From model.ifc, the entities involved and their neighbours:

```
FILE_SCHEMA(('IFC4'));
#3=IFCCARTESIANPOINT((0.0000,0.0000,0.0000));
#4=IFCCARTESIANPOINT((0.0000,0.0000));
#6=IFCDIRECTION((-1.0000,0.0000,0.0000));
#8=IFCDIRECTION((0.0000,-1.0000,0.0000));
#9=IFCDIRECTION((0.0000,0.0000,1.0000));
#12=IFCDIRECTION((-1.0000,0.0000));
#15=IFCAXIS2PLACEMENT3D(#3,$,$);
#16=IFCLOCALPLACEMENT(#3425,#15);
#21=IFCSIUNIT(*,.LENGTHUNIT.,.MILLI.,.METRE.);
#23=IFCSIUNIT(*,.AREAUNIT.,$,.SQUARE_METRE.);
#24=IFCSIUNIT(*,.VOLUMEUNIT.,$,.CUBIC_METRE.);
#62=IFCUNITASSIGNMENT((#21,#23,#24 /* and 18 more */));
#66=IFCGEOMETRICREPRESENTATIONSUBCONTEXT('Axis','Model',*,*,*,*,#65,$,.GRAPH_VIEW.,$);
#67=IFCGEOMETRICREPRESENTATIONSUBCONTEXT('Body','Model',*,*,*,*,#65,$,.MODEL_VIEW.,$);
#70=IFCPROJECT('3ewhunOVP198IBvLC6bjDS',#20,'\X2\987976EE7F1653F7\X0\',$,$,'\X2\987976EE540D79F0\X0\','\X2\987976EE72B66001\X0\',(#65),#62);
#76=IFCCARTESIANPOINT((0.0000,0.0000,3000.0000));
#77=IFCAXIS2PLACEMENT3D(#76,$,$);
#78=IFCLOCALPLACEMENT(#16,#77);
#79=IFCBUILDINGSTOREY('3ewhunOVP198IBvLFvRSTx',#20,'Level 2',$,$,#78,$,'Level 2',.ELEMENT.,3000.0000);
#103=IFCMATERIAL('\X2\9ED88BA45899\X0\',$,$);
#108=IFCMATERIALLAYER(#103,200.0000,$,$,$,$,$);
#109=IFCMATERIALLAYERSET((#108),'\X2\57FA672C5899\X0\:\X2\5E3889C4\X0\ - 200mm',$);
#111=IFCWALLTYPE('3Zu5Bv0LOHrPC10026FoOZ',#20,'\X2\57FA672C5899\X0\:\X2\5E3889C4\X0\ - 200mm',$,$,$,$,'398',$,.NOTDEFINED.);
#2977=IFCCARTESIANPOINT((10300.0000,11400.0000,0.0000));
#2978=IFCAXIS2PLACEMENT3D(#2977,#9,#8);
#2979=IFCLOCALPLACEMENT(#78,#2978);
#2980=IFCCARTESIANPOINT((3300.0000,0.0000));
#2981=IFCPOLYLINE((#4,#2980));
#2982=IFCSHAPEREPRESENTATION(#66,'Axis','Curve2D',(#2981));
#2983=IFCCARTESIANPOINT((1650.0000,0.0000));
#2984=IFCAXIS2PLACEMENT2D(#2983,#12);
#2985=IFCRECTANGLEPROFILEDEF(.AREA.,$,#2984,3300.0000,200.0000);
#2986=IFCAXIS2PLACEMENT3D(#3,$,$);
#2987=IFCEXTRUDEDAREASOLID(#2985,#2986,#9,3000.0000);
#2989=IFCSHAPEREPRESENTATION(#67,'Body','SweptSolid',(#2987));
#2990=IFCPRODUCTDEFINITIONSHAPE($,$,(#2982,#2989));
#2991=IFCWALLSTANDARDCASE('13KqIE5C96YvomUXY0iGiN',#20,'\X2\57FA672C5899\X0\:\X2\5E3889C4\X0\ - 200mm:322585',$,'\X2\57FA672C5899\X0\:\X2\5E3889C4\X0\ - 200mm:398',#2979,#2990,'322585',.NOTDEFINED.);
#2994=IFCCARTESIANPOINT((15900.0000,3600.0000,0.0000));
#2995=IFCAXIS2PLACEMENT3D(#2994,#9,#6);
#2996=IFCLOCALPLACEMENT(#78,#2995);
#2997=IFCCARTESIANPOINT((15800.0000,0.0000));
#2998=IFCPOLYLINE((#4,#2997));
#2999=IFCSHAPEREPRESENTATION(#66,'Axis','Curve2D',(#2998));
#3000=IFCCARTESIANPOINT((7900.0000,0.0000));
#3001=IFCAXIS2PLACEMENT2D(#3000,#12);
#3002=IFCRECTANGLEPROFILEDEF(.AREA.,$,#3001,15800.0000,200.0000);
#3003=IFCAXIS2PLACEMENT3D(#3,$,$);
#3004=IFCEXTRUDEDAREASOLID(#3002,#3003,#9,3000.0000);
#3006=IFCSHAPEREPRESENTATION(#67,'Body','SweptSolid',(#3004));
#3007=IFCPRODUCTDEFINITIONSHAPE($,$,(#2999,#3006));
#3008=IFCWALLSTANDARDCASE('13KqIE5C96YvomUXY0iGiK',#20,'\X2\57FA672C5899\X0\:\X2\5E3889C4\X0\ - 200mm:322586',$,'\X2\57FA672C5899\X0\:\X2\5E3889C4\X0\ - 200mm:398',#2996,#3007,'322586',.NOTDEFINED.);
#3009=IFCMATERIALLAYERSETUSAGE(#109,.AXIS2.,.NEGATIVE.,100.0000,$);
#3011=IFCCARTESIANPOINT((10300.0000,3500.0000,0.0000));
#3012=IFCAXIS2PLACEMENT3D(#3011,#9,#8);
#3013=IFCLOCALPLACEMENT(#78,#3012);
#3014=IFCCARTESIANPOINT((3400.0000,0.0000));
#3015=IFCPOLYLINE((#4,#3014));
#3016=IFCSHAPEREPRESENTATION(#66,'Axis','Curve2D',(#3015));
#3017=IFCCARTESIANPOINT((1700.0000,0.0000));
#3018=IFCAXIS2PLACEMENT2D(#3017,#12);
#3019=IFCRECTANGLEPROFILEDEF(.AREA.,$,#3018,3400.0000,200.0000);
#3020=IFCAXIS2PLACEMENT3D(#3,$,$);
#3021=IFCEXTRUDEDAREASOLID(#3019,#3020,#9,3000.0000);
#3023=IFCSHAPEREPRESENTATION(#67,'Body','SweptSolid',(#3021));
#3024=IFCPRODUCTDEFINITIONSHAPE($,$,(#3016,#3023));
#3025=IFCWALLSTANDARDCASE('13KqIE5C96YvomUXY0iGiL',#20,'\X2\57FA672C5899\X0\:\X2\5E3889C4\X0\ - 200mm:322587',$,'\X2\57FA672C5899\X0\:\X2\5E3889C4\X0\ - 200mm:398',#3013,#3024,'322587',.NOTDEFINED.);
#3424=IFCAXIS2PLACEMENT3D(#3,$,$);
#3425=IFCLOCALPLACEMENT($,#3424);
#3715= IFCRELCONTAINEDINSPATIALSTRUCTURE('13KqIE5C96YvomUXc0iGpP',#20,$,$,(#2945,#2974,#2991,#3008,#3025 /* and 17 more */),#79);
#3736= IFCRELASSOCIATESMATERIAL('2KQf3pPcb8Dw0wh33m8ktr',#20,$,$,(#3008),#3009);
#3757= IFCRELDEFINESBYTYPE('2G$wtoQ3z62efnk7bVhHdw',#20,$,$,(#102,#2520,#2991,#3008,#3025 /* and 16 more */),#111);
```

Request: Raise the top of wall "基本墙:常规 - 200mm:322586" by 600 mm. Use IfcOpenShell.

```python
import ifcopenshell
import ifcopenshell.geom
import ifcopenshell.util.representation
import ifcopenshell.util.shape
import ifcopenshell.util.unit

model = ifcopenshell.open("model.ifc")
unit_scale = ifcopenshell.util.unit.calculate_unit_scale(model)
settings = ifcopenshell.geom.settings()


def volume(element):
    """Net volume in cubic metres, openings subtracted."""
    shape = ifcopenshell.geom.create_shape(settings, element)
    return ifcopenshell.util.shape.get_volume(shape.geometry)


wall = model.by_guid("13KqIE5C96YvomUXY0iGiK")
before = volume(wall)

body = ifcopenshell.util.representation.get_representation(wall, "Model", "Body")
solid = body.Items[0]
old_height = solid.Depth
solid.Depth += 0.6 / unit_scale
after = volume(wall)

print(f"height {old_height:g} -> {solid.Depth:g}, volume {before:.3f} -> {after:.3f} m3")

model.write("model_updated.ifc")
```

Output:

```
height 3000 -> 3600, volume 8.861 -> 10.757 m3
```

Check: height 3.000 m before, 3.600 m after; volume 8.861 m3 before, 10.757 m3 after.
